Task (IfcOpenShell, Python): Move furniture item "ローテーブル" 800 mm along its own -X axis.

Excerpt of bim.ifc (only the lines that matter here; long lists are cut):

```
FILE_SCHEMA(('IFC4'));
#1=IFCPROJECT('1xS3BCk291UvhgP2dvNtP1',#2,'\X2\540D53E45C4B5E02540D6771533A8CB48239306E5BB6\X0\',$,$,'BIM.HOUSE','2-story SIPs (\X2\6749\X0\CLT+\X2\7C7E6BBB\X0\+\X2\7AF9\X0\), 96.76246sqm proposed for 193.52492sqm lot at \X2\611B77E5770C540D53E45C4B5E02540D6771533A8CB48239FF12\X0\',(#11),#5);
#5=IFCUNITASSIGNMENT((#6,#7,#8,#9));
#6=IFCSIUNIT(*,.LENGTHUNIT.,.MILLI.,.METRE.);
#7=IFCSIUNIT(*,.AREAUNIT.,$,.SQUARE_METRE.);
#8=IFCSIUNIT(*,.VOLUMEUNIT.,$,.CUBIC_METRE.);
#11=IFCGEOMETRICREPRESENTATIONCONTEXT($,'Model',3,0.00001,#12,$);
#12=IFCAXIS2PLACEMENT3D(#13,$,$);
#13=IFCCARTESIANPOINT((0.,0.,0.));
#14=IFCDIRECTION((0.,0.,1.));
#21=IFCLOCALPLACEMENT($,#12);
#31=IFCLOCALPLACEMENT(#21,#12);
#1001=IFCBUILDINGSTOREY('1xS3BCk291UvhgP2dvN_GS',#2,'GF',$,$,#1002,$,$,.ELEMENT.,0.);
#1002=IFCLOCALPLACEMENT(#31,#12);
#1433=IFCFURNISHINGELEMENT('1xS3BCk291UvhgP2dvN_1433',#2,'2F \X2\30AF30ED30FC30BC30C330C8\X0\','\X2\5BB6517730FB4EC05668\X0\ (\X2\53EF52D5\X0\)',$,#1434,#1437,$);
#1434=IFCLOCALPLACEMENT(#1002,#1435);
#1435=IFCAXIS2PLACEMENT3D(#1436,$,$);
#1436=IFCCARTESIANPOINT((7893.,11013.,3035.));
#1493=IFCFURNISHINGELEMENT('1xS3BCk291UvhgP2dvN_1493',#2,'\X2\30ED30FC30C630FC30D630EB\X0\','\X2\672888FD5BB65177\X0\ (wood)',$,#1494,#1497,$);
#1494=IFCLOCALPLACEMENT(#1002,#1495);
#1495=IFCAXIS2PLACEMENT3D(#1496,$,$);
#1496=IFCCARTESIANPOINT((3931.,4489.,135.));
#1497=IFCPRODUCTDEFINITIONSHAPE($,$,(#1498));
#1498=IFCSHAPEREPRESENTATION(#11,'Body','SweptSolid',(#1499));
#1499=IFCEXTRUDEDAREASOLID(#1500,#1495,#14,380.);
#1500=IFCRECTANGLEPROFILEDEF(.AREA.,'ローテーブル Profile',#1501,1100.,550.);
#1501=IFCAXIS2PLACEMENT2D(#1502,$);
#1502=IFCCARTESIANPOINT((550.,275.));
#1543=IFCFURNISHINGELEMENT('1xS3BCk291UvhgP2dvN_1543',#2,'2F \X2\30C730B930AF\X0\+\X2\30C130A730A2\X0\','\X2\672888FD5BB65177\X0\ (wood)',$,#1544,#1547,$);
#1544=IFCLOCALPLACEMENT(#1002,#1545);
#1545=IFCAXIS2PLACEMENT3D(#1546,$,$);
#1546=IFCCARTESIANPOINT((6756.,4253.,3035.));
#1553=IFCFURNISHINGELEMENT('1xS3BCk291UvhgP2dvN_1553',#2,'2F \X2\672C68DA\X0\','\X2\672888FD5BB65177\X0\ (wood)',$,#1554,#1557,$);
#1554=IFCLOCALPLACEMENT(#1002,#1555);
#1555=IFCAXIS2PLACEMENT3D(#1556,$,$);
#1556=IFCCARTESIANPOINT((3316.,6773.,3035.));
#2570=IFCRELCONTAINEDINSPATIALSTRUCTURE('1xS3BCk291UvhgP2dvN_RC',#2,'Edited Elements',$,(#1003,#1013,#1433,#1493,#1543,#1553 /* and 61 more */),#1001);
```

```python
import ifcopenshell
import ifcopenshell.api.geometry
import ifcopenshell.util.placement
import ifcopenshell.util.unit

model = ifcopenshell.open("bim.ifc")
unit_scale = ifcopenshell.util.unit.calculate_unit_scale(model)

item = model.by_guid("1xS3BCk291UvhgP2dvN_1493")
matrix = ifcopenshell.util.placement.get_local_placement(item.ObjectPlacement)
matrix[:3, 3] -= matrix[:3, 0] * 0.8 / unit_scale
ifcopenshell.api.geometry.edit_object_placement(model, product=item, matrix=matrix, is_si=False)

print(ifcopenshell.util.placement.get_local_placement(item.ObjectPlacement).round(3) + 0.0)

model.write("bim-out.ifc")
```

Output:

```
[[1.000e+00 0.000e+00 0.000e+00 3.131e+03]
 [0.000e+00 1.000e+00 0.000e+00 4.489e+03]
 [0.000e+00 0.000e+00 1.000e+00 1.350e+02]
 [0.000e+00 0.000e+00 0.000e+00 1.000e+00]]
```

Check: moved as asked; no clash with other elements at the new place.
